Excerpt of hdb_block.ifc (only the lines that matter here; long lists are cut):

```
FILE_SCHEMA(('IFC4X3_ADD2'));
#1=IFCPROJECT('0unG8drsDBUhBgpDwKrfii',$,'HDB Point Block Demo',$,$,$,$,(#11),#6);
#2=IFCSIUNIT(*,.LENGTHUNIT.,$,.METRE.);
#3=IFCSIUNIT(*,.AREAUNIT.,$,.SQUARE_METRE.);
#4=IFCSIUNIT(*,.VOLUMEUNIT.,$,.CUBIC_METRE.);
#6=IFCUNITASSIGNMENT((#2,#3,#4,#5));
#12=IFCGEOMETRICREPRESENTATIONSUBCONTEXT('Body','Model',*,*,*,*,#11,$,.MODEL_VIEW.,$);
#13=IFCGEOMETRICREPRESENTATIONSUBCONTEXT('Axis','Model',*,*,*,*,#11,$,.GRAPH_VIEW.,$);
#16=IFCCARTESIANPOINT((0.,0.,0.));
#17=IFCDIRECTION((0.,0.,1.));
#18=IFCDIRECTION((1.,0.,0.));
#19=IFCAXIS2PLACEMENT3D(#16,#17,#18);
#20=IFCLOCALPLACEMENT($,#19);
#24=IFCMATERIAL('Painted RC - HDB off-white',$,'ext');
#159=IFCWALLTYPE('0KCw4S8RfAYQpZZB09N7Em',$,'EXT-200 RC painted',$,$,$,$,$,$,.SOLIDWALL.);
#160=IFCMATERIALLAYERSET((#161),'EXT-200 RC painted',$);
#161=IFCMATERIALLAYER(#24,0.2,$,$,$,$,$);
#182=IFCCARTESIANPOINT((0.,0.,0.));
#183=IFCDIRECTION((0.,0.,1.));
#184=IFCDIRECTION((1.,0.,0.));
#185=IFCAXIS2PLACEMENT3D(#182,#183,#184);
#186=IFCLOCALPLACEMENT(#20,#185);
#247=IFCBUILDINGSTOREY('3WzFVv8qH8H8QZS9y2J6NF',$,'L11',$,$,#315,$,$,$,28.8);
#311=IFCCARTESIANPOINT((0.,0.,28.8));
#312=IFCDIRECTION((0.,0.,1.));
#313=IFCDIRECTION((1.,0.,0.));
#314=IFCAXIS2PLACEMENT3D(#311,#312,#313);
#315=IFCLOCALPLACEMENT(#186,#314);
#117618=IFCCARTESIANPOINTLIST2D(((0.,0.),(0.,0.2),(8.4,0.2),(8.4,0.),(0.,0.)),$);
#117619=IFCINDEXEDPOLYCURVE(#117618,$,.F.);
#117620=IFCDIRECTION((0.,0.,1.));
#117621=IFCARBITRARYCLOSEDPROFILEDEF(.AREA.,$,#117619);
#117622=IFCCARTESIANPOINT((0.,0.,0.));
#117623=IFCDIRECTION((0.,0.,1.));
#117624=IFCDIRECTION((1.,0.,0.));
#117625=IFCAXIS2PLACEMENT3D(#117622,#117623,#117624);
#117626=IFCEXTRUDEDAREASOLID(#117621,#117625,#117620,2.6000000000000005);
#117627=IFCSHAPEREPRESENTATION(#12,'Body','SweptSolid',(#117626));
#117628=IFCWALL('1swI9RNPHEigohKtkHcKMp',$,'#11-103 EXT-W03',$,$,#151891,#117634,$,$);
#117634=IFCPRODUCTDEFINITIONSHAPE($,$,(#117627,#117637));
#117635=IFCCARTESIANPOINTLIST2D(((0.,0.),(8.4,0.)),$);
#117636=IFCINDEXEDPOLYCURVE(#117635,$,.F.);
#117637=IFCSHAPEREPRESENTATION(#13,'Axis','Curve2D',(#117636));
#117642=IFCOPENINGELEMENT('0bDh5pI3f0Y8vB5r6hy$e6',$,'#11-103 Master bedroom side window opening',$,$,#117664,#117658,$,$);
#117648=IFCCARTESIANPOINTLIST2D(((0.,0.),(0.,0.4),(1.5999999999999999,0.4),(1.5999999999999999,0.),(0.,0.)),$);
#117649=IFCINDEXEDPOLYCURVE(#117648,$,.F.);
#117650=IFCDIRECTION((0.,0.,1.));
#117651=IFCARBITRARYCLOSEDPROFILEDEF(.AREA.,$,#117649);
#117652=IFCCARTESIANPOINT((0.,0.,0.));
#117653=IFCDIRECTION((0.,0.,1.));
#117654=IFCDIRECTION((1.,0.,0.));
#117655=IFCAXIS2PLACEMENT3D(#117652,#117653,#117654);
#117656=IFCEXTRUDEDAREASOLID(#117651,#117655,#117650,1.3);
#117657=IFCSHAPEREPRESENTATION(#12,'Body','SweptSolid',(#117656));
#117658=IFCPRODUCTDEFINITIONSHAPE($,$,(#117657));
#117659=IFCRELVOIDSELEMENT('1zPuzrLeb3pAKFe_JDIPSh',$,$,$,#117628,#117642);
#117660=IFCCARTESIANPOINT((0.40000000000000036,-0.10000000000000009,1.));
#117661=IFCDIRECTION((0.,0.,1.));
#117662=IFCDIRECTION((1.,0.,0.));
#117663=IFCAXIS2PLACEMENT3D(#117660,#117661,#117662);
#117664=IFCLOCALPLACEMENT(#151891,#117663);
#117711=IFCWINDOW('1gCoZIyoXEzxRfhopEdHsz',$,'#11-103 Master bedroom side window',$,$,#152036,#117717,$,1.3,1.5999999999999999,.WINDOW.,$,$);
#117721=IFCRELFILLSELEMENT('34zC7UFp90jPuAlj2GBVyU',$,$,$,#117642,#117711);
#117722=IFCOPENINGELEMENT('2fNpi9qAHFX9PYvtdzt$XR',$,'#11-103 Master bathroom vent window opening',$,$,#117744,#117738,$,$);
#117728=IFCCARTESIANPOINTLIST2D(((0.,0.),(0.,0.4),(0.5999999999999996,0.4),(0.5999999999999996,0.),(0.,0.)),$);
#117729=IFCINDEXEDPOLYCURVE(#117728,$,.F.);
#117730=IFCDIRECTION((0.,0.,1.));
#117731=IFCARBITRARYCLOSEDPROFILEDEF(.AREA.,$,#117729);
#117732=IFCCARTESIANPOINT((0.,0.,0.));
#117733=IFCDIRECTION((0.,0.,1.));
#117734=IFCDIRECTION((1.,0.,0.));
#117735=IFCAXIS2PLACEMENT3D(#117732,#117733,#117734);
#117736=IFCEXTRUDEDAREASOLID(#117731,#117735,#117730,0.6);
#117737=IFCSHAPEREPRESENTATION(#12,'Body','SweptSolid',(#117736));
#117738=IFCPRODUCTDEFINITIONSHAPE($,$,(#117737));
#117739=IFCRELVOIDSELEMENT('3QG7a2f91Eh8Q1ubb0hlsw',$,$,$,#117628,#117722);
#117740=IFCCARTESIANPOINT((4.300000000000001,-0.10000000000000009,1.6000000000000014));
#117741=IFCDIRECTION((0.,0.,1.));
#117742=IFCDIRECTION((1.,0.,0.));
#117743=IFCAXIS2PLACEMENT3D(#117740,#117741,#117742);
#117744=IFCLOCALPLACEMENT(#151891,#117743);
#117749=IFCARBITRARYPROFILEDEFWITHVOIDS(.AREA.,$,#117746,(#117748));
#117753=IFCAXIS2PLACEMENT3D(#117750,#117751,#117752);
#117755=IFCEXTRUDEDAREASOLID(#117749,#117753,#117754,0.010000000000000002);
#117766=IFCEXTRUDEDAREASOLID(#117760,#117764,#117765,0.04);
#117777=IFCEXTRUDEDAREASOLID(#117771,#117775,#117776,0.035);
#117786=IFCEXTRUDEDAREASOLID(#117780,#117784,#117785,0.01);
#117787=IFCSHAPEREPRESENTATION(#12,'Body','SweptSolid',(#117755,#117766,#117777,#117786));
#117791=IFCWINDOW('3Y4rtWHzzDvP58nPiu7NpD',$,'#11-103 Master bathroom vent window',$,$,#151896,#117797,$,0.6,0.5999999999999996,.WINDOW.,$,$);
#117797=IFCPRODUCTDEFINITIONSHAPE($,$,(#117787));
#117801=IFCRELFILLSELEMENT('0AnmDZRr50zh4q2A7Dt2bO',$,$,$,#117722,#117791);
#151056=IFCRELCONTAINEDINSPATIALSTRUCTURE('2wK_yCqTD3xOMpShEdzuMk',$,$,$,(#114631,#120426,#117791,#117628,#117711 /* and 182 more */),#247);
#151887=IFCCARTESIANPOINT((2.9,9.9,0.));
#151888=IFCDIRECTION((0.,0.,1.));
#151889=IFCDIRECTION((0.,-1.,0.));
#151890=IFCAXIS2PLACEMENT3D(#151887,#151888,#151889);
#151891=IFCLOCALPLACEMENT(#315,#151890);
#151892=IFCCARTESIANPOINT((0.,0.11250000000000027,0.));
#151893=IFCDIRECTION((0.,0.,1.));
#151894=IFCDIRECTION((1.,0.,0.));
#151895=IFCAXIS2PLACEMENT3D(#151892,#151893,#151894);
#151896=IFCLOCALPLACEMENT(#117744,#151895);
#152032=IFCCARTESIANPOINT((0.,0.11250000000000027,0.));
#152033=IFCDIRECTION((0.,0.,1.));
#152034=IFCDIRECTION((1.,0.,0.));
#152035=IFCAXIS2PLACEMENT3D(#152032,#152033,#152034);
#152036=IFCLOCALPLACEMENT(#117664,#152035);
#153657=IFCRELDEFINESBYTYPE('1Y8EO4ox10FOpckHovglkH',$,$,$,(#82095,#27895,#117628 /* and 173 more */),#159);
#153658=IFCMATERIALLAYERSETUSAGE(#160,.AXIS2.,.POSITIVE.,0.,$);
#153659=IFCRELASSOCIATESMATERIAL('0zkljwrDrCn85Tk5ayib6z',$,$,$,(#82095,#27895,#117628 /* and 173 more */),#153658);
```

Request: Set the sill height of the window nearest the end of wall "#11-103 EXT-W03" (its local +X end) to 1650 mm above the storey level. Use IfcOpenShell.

```python
import numpy as np
import ifcopenshell
import ifcopenshell.api.geometry
import ifcopenshell.geom
import ifcopenshell.util.element
import ifcopenshell.util.placement
import ifcopenshell.util.shape
import ifcopenshell.util.unit

model = ifcopenshell.open("hdb_block.ifc")
unit_scale = ifcopenshell.util.unit.calculate_unit_scale(model)

window = model.by_guid("3Y4rtWHzzDvP58nPiu7NpD")
opening = window.FillsVoids[0].RelatingOpeningElement
storey = ifcopenshell.util.element.get_container(window, ifc_class="IfcBuildingStorey")
level = ifcopenshell.util.placement.get_local_placement(storey.ObjectPlacement)[2, 3]

# The opening's origin need not be at the sill, so measure its lowest point.
shape = ifcopenshell.geom.create_shape(ifcopenshell.geom.settings(), opening)
bottom = ifcopenshell.util.shape.get_shape_bottom_elevation(shape, shape.geometry) / unit_scale
dz = level + 1.65 / unit_scale - bottom

shift = np.array([0.0, 0.0, dz])
# The window is placed relative to its opening, so it follows when the opening moves.
matrix = ifcopenshell.util.placement.get_local_placement(opening.ObjectPlacement)
matrix[:3, 3] += shift
ifcopenshell.api.geometry.edit_object_placement(
    model, product=opening, matrix=matrix, is_si=False, should_transform_children=True
)

print(f"moved by {dz * unit_scale:+.3f} m")

model.write("hdb_block_edited.ifc")
```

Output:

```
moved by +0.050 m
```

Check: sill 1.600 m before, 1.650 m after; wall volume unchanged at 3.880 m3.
